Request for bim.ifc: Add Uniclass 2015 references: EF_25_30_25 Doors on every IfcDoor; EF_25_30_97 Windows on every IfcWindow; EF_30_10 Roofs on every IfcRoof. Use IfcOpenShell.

First a look at what the model holds.

```python
import ifcopenshell

model = ifcopenshell.open("bim.ifc")
print(model.schema)
print("classifications:", [c.Name for c in model.by_type("IfcClassification")])
for ifc_class in ("IfcDoor", "IfcRoof", "IfcStair", "IfcWall", "IfcWindow"):
    print(ifc_class, len(model.by_type(ifc_class)))
```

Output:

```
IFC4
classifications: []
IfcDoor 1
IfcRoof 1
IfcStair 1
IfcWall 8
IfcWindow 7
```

```python
import ifcopenshell
import ifcopenshell.api.classification

model = ifcopenshell.open("bim.ifc")

system = ifcopenshell.api.classification.add_classification(model, classification="Uniclass 2015")

codes = {
    "IfcDoor": ("EF_25_30_25", "Doors"),
    "IfcWindow": ("EF_25_30_97", "Windows"),
    "IfcRoof": ("EF_30_10", "Roofs"),
}
for ifc_class, (code, name) in codes.items():
    products = model.by_type(ifc_class)
    ifcopenshell.api.classification.add_reference(
        model, products=products, classification=system, identification=code, name=name
    )
    print(code, len(products))

model.write("bim_v2.ifc")
```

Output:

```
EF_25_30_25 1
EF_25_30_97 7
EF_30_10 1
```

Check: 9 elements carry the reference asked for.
